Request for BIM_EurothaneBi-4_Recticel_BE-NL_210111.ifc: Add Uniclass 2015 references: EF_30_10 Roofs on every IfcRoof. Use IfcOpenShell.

First a look at what the model holds.

```python
import ifcopenshell

model = ifcopenshell.open("BIM_EurothaneBi-4_Recticel_BE-NL_210111.ifc")
print(model.schema)
print("classifications:", [c.Name for c in model.by_type("IfcClassification")])
for ifc_class in ("IfcDoor", "IfcRoof", "IfcStair", "IfcWall", "IfcWindow"):
    print(ifc_class, len(model.by_type(ifc_class)))
```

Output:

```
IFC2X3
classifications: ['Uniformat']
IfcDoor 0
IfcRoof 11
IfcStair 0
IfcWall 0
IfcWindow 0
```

```python
import ifcopenshell
import ifcopenshell.api.classification

model = ifcopenshell.open("BIM_EurothaneBi-4_Recticel_BE-NL_210111.ifc")

# IFC2X3 requires Source and Edition and has no link from the project to the system.
system = model.create_entity("IfcClassification", Source="NBS", Edition="2015", Name="Uniclass 2015")

codes = {
    "IfcRoof": ("EF_30_10", "Roofs"),
}
for ifc_class, (code, name) in codes.items():
    products = model.by_type(ifc_class)
    ifcopenshell.api.classification.add_reference(
        model, products=products, classification=system, identification=code, name=name
    )
    print(code, len(products))

model.write("BIM_EurothaneBi-4_Recticel_BE-NL_210111-out.ifc")
```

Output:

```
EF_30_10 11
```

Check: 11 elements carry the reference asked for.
